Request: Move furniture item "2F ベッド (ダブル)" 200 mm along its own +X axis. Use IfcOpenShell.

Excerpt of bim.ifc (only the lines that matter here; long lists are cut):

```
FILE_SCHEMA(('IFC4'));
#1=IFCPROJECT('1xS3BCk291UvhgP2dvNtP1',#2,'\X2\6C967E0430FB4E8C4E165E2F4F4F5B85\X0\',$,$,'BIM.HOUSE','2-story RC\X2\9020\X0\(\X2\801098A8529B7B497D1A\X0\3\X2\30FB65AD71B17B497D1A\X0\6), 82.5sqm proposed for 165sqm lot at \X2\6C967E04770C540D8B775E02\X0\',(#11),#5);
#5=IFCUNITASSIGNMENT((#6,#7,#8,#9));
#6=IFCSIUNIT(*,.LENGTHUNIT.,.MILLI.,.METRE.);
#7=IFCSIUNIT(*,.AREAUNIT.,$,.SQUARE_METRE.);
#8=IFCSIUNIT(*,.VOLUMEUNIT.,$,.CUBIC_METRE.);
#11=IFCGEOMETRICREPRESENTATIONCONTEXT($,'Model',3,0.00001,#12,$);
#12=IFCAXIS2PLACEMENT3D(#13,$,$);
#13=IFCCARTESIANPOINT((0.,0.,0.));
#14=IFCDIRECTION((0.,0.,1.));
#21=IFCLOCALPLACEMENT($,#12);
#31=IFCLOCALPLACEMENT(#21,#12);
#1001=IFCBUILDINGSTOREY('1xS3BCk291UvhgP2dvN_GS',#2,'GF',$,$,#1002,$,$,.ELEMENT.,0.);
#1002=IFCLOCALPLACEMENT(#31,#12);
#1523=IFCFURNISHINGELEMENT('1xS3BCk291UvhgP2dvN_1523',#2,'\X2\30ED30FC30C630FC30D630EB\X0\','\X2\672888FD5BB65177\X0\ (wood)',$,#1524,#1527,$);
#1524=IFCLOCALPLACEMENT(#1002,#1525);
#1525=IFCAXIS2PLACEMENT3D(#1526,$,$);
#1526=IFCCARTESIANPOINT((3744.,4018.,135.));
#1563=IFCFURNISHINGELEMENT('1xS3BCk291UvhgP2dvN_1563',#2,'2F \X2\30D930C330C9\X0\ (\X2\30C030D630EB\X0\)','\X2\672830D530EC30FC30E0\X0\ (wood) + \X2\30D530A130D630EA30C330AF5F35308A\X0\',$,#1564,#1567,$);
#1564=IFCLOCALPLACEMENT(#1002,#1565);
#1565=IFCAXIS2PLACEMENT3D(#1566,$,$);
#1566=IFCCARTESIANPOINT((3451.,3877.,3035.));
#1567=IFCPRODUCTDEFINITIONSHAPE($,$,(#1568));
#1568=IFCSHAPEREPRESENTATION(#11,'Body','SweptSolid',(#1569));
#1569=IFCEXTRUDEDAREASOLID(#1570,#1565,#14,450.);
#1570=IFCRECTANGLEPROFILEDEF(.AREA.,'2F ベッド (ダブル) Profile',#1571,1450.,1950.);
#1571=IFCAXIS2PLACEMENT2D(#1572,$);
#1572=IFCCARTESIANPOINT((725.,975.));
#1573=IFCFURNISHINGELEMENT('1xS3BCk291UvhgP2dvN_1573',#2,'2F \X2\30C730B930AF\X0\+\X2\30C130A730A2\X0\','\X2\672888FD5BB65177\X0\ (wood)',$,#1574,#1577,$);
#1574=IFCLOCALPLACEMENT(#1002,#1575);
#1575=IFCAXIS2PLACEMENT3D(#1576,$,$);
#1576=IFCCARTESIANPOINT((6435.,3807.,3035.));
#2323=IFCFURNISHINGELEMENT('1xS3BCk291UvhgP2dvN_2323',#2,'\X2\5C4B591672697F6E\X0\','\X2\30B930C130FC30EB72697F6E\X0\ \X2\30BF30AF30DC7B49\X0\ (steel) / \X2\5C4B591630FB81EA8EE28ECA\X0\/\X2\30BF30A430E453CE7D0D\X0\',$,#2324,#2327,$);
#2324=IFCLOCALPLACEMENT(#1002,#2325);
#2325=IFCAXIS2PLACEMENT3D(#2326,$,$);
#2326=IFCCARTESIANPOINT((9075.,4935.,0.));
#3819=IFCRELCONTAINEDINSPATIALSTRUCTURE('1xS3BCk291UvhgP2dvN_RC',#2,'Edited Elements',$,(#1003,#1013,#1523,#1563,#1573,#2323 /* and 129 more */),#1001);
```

```python
import ifcopenshell
import ifcopenshell.api.geometry
import ifcopenshell.util.placement
import ifcopenshell.util.unit

model = ifcopenshell.open("bim.ifc")
unit_scale = ifcopenshell.util.unit.calculate_unit_scale(model)

item = model.by_id(1563)
matrix = ifcopenshell.util.placement.get_local_placement(item.ObjectPlacement)
matrix[:3, 3] += matrix[:3, 0] * 0.2 / unit_scale
ifcopenshell.api.geometry.edit_object_placement(model, product=item, matrix=matrix, is_si=False)

print(ifcopenshell.util.placement.get_local_placement(item.ObjectPlacement).round(3) + 0.0)

model.write("bim_edited.ifc")
```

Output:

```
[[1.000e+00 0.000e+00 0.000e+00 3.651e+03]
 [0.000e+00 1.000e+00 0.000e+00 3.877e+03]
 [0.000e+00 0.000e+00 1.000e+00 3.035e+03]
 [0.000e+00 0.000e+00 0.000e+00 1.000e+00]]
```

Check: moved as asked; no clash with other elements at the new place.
